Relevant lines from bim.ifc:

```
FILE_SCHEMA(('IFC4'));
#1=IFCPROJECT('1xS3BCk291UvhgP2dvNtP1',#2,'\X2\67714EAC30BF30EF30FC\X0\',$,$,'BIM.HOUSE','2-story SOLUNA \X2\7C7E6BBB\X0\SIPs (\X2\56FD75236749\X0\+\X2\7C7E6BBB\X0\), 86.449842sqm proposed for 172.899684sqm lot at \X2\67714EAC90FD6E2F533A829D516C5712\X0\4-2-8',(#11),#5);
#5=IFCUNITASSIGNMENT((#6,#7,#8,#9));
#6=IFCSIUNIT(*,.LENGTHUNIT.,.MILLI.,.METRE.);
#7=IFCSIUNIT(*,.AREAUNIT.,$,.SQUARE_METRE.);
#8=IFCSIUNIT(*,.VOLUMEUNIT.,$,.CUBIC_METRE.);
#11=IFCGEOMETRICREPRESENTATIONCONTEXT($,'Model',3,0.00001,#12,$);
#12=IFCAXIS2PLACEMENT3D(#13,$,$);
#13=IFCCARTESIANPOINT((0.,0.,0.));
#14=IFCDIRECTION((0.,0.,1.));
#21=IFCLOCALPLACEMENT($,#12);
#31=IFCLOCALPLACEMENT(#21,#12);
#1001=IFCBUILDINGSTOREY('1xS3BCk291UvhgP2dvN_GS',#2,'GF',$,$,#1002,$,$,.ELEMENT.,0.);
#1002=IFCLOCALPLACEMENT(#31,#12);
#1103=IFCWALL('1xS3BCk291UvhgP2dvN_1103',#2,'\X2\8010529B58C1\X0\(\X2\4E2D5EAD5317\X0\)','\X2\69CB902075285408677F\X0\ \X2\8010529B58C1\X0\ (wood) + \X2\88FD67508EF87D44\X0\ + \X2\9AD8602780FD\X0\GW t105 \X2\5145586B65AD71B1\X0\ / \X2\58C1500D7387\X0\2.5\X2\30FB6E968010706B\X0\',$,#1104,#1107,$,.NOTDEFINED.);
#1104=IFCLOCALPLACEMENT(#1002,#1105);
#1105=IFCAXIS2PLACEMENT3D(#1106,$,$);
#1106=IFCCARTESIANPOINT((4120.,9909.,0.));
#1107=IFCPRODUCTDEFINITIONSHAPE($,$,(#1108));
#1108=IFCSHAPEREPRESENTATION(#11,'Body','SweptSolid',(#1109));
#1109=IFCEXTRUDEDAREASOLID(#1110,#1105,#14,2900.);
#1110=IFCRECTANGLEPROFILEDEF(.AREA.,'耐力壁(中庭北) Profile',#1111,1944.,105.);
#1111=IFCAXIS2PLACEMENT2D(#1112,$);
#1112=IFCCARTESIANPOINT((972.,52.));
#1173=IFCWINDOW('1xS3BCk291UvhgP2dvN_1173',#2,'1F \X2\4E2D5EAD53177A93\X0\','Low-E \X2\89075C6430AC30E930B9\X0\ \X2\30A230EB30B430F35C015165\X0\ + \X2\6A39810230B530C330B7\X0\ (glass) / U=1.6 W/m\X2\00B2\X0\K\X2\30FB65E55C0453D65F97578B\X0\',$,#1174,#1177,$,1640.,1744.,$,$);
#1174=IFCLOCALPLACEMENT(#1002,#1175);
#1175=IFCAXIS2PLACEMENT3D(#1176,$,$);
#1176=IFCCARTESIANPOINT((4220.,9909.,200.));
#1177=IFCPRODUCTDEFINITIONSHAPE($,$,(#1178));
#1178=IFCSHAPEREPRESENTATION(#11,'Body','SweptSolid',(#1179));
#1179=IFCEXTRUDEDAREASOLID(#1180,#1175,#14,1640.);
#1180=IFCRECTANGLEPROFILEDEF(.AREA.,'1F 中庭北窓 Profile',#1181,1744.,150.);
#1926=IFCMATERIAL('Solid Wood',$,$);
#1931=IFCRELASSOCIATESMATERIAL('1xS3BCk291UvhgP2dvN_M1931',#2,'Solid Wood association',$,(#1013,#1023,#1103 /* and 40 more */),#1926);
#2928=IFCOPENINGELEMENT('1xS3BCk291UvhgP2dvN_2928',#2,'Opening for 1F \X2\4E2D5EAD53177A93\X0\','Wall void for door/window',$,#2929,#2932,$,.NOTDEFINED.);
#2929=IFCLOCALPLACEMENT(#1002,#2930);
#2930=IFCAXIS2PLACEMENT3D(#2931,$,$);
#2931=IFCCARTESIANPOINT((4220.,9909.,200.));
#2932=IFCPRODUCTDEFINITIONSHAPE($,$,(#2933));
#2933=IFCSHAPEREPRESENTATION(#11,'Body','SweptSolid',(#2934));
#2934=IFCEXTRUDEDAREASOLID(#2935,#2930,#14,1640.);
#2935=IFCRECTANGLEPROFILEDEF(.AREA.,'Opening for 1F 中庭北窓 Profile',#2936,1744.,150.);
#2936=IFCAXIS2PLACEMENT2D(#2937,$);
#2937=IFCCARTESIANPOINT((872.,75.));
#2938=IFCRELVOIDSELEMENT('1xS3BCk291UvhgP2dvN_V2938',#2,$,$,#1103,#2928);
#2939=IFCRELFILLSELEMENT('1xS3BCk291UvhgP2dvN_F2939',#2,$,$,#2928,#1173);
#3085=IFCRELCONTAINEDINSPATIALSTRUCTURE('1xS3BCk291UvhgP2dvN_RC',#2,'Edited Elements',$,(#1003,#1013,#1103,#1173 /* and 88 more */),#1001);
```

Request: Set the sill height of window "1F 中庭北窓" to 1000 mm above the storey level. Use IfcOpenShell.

```python
import numpy as np
import ifcopenshell
import ifcopenshell.api.geometry
import ifcopenshell.geom
import ifcopenshell.util.element
import ifcopenshell.util.placement
import ifcopenshell.util.shape
import ifcopenshell.util.unit

model = ifcopenshell.open("bim.ifc")
unit_scale = ifcopenshell.util.unit.calculate_unit_scale(model)

window = model.by_guid("1xS3BCk291UvhgP2dvN_1173")
opening = window.FillsVoids[0].RelatingOpeningElement
storey = ifcopenshell.util.element.get_container(window, ifc_class="IfcBuildingStorey")
level = ifcopenshell.util.placement.get_local_placement(storey.ObjectPlacement)[2, 3]

# The opening's origin need not be at the sill, so measure its lowest point.
shape = ifcopenshell.geom.create_shape(ifcopenshell.geom.settings(), opening)
bottom = ifcopenshell.util.shape.get_shape_bottom_elevation(shape, shape.geometry) / unit_scale
dz = level + 1 / unit_scale - bottom

shift = np.array([0.0, 0.0, dz])
# The window is not placed relative to its opening, so move both.
for product in (opening, window):
    matrix = ifcopenshell.util.placement.get_local_placement(product.ObjectPlacement)
    matrix[:3, 3] += shift
    ifcopenshell.api.geometry.edit_object_placement(model, product=product, matrix=matrix, is_si=False)

print(f"moved by {dz * unit_scale:+.3f} m")

model.write("bim_edited.ifc")
```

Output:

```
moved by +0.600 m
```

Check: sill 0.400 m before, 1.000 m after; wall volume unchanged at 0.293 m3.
